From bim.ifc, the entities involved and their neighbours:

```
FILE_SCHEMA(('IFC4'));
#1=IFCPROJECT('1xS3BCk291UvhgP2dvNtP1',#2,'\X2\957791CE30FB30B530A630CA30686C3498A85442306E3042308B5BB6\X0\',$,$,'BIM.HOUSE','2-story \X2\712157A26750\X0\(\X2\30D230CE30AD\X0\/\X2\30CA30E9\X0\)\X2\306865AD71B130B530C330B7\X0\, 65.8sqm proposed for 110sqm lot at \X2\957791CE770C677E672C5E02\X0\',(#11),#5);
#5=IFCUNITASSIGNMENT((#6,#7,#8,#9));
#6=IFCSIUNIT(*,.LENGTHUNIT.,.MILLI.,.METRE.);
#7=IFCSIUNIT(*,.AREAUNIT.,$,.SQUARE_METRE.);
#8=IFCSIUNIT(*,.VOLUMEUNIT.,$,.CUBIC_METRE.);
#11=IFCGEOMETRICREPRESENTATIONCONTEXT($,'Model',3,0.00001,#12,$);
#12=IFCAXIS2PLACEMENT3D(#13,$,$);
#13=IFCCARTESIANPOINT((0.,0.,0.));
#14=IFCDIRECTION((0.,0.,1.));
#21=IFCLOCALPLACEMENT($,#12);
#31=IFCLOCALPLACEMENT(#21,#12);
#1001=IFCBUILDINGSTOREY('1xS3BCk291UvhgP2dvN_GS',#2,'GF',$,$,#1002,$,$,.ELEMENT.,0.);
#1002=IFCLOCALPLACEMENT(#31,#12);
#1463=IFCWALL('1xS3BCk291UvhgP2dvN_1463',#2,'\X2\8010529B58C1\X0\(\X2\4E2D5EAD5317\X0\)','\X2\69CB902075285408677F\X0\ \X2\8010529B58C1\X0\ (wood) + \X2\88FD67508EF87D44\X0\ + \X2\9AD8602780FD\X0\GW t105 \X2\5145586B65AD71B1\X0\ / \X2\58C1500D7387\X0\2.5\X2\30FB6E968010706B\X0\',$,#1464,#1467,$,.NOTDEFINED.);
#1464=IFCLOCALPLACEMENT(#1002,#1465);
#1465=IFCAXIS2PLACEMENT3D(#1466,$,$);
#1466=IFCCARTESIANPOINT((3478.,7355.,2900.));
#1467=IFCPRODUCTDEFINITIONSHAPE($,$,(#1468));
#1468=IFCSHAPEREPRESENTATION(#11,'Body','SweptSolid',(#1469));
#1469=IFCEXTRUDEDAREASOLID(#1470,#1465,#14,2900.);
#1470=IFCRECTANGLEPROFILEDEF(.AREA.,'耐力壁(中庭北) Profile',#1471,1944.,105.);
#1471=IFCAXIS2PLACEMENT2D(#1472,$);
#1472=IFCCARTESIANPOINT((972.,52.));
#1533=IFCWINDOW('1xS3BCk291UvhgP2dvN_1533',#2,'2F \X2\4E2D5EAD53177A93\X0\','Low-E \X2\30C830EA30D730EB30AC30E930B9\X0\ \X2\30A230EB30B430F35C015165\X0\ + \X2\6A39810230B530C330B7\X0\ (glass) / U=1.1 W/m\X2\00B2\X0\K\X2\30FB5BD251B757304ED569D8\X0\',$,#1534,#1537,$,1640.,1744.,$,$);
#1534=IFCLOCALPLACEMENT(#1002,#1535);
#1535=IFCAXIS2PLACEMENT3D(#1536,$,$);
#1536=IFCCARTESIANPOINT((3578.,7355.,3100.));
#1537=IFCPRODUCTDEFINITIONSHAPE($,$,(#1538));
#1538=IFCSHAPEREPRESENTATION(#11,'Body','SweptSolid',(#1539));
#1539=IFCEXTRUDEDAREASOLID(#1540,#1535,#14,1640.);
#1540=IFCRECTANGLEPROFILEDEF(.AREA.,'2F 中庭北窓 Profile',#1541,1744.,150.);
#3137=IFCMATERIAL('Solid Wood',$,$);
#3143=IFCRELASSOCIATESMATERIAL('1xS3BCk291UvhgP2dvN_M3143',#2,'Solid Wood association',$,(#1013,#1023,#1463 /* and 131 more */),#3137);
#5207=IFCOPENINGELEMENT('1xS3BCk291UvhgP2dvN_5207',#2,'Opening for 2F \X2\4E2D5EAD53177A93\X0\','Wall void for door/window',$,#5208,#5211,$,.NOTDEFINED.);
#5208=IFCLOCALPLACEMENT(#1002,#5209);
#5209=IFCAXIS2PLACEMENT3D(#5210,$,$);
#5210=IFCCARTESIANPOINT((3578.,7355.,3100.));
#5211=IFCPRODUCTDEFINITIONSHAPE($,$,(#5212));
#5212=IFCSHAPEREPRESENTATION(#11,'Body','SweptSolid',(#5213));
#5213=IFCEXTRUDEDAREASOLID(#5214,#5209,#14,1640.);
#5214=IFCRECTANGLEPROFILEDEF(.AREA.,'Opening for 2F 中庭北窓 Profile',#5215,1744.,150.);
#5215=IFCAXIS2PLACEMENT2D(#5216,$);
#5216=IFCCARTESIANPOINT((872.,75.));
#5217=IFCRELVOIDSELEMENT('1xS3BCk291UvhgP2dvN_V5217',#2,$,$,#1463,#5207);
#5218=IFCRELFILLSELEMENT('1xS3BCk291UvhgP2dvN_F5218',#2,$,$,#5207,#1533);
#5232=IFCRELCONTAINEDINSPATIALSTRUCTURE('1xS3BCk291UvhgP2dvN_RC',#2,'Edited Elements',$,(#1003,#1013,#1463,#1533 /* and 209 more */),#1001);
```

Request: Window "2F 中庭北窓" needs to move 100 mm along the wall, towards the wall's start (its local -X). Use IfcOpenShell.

```python
import ifcopenshell
import ifcopenshell.api.geometry
import ifcopenshell.util.placement
import ifcopenshell.util.unit

model = ifcopenshell.open("bim.ifc")
unit_scale = ifcopenshell.util.unit.calculate_unit_scale(model)

window = model.by_guid("1xS3BCk291UvhgP2dvN_1533")
opening = window.FillsVoids[0].RelatingOpeningElement
wall = opening.VoidsElements[0].RelatingBuildingElement

wall_matrix = ifcopenshell.util.placement.get_local_placement(wall.ObjectPlacement)
shift = wall_matrix[:3, 0] * -0.1 / unit_scale
before = ifcopenshell.util.placement.get_local_placement(window.ObjectPlacement)[:3, 3].copy()

# The window is not placed relative to its opening, so move both.
for product in (opening, window):
    matrix = ifcopenshell.util.placement.get_local_placement(product.ObjectPlacement)
    matrix[:3, 3] += shift
    ifcopenshell.api.geometry.edit_object_placement(model, product=product, matrix=matrix, is_si=False)

after = ifcopenshell.util.placement.get_local_placement(window.ObjectPlacement)[:3, 3]
print("window moved by", (after - before).round(3) + 0.0)

model.write("bim_v2.ifc")
```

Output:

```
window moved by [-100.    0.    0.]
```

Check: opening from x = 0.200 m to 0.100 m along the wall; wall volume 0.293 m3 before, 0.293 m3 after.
